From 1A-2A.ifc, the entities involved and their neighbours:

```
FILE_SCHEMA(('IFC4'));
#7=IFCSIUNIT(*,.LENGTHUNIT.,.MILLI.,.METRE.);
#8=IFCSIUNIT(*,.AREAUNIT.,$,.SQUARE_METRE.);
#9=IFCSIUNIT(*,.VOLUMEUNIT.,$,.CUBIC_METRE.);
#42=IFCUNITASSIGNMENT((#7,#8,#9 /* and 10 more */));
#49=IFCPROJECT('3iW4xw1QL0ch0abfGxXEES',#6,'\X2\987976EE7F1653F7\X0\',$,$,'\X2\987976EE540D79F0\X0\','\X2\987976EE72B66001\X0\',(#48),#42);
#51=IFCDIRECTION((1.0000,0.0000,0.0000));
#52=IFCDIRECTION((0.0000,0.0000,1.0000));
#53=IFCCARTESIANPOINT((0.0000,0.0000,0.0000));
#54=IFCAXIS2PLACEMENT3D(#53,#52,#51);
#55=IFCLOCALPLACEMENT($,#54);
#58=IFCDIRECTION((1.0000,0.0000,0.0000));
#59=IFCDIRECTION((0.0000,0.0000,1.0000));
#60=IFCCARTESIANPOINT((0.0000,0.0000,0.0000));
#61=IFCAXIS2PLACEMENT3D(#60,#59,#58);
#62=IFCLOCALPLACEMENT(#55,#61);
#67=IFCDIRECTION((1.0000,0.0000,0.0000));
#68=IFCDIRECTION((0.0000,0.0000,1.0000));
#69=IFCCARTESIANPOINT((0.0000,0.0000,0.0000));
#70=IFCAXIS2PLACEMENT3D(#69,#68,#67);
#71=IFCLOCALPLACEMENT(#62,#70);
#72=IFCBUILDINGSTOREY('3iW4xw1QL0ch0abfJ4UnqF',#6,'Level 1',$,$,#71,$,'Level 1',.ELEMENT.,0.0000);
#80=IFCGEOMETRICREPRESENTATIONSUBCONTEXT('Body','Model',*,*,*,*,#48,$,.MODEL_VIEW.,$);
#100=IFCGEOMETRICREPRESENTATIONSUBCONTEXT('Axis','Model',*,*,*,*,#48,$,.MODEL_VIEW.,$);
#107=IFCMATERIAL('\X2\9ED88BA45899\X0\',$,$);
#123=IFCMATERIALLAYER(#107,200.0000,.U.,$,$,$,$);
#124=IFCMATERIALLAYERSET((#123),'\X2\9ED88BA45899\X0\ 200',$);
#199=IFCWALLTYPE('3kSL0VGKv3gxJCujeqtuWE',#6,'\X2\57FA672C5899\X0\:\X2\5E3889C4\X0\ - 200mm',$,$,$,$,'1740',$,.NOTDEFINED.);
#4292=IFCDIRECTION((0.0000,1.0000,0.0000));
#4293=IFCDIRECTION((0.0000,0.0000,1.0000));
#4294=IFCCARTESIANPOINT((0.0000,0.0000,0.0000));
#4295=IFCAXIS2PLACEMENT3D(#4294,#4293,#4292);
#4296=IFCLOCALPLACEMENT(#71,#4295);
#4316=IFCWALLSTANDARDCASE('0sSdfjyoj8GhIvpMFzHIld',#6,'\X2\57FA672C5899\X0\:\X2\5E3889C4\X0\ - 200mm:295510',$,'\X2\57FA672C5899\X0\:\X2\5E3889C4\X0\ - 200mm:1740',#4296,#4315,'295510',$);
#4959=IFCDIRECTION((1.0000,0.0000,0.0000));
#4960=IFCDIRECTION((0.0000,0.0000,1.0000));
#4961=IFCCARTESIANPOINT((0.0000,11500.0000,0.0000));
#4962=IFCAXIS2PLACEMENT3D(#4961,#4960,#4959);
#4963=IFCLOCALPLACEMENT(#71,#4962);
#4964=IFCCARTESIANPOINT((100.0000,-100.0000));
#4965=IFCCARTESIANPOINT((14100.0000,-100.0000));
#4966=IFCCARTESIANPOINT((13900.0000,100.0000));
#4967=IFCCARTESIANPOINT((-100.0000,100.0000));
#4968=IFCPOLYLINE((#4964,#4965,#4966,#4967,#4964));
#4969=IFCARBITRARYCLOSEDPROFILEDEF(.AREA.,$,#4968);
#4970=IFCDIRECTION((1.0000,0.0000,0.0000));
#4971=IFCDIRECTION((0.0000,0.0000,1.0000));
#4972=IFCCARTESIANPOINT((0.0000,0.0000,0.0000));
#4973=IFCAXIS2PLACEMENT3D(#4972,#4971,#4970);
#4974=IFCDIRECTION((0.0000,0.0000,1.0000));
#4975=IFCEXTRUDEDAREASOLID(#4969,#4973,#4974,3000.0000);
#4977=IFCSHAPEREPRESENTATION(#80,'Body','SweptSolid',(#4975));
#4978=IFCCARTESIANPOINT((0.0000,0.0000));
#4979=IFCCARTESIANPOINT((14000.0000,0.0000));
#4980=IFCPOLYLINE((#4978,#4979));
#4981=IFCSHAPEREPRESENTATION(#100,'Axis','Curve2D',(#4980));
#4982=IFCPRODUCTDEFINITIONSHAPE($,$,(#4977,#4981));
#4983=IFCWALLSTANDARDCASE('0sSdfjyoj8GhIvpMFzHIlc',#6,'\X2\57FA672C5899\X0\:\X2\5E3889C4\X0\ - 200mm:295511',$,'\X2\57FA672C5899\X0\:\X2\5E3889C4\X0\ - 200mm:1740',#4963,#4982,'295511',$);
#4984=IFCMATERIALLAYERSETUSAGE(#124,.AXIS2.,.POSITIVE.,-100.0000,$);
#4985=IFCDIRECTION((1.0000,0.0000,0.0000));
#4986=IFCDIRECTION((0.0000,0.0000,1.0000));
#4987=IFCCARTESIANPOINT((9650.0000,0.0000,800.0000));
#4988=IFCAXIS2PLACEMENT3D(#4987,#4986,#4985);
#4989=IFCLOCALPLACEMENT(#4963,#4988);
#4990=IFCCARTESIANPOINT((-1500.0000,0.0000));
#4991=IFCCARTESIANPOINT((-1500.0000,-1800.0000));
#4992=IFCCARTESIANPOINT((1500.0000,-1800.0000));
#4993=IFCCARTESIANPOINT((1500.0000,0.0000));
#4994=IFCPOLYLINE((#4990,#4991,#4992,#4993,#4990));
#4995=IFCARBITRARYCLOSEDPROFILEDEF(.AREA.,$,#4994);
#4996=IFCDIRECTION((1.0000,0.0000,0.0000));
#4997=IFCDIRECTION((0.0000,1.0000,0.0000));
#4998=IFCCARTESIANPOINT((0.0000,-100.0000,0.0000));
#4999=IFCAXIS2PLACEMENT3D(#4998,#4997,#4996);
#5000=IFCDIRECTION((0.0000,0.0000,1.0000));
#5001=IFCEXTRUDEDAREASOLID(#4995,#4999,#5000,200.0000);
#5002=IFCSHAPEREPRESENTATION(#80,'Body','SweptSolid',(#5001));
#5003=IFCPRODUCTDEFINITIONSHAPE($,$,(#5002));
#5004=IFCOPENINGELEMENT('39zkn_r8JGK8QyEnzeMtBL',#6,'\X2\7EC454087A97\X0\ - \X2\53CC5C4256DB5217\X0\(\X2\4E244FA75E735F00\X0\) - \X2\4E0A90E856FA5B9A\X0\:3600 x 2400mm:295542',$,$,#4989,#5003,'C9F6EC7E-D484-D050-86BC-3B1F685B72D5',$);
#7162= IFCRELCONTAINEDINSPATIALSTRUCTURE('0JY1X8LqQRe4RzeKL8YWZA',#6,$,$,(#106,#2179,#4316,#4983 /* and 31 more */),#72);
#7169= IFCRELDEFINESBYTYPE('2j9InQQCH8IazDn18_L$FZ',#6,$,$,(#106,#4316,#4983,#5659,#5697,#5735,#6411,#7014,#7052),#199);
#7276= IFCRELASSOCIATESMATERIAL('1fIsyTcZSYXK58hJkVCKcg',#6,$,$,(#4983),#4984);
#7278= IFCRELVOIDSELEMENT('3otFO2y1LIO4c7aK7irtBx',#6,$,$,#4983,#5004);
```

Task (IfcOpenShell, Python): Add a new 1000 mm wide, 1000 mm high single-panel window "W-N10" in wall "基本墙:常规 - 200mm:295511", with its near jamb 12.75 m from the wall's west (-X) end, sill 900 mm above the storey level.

```python
import numpy as np
import ifcopenshell
import ifcopenshell.api.feature
import ifcopenshell.api.geometry
import ifcopenshell.api.root
import ifcopenshell.api.spatial
import ifcopenshell.geom
import ifcopenshell.util.element
import ifcopenshell.util.placement
import ifcopenshell.util.representation
import ifcopenshell.util.shape
import ifcopenshell.util.unit

model = ifcopenshell.open("1A-2A.ifc")
unit_scale = ifcopenshell.util.unit.calculate_unit_scale(model)
settings = ifcopenshell.geom.settings()


def volume(element):
    """Net volume in cubic metres, openings subtracted."""
    shape = ifcopenshell.geom.create_shape(settings, element)
    return ifcopenshell.util.shape.get_volume(shape.geometry)


wall = model.by_guid("0sSdfjyoj8GhIvpMFzHIlc")
storey = ifcopenshell.util.element.get_container(wall, ifc_class="IfcBuildingStorey")
context = ifcopenshell.util.representation.get_context(model, "Model", "Body", "MODEL_VIEW")
before = volume(wall)

width, height, from_end, sill = 1, 1, 12.75, 0.9  # metres

# The wall runs along its own X axis, and the end named is its -X end.
wall_shape = ifcopenshell.geom.create_shape(settings, wall)
x, y, z = ifcopenshell.util.shape.get_vertices(wall_shape.geometry).T
start = x.min() + from_end
face, thickness = float(y.min()), float(y.max() - y.min())
wall_matrix = ifcopenshell.util.placement.get_local_placement(wall.ObjectPlacement)
level = ifcopenshell.util.placement.get_local_placement(storey.ObjectPlacement)[2, 3]


def in_wall(x, y):
    """Placement at x, y metres in the wall's axes, at sill height."""
    matrix = wall_matrix.copy()
    matrix[:, 3] = wall_matrix @ np.array([x / unit_scale, y / unit_scale, 0.0, 1.0])
    matrix[2, 3] = level + sill / unit_scale
    return matrix


# Opening: a box that overshoots both wall faces by 50 mm.
opening = ifcopenshell.api.root.create_entity(model, ifc_class="IfcOpeningElement", predefined_type="OPENING")
box = ifcopenshell.api.geometry.add_wall_representation(
    model, context=context, length=width, height=height, thickness=thickness + 0.1
)
ifcopenshell.api.geometry.assign_representation(model, product=opening, representation=box)
ifcopenshell.api.geometry.edit_object_placement(model, product=opening, matrix=in_wall(start, face - 0.05), is_si=False)
ifcopenshell.api.feature.add_feature(model, feature=opening, element=wall)

window = ifcopenshell.api.root.create_entity(model, ifc_class="IfcWindow", name="W-N10", predefined_type="WINDOW")
window.OverallWidth, window.OverallHeight = width / unit_scale, height / unit_scale
window.PartitioningType = "SINGLE_PANEL"
body = ifcopenshell.api.geometry.add_window_representation(
    model,
    context=context,
    overall_width=window.OverallWidth,
    overall_height=window.OverallHeight,
    partition_type="SINGLE_PANEL",
)
ifcopenshell.api.geometry.assign_representation(model, product=window, representation=body)
ifcopenshell.api.spatial.assign_container(model, products=[window], relating_structure=storey)
ifcopenshell.api.feature.add_filling(model, opening=opening, element=window)

# Centre the window in the wall's thickness.
ifcopenshell.api.geometry.edit_object_placement(model, product=window, matrix=in_wall(start, face), is_si=False)
window_shape = ifcopenshell.geom.create_shape(settings, window)
depth = ifcopenshell.util.shape.get_vertices(window_shape.geometry)[:, 1]
offset = face + thickness / 2 - (depth.min() + depth.max()) / 2
ifcopenshell.api.geometry.edit_object_placement(model, product=window, matrix=in_wall(start, offset), is_si=False)

after = volume(wall)

print(f"wall volume {before:.3f} -> {after:.3f} m3")

model.write("1A-2A_rev.ifc")
```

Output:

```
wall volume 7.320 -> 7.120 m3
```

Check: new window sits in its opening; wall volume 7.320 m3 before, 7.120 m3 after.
